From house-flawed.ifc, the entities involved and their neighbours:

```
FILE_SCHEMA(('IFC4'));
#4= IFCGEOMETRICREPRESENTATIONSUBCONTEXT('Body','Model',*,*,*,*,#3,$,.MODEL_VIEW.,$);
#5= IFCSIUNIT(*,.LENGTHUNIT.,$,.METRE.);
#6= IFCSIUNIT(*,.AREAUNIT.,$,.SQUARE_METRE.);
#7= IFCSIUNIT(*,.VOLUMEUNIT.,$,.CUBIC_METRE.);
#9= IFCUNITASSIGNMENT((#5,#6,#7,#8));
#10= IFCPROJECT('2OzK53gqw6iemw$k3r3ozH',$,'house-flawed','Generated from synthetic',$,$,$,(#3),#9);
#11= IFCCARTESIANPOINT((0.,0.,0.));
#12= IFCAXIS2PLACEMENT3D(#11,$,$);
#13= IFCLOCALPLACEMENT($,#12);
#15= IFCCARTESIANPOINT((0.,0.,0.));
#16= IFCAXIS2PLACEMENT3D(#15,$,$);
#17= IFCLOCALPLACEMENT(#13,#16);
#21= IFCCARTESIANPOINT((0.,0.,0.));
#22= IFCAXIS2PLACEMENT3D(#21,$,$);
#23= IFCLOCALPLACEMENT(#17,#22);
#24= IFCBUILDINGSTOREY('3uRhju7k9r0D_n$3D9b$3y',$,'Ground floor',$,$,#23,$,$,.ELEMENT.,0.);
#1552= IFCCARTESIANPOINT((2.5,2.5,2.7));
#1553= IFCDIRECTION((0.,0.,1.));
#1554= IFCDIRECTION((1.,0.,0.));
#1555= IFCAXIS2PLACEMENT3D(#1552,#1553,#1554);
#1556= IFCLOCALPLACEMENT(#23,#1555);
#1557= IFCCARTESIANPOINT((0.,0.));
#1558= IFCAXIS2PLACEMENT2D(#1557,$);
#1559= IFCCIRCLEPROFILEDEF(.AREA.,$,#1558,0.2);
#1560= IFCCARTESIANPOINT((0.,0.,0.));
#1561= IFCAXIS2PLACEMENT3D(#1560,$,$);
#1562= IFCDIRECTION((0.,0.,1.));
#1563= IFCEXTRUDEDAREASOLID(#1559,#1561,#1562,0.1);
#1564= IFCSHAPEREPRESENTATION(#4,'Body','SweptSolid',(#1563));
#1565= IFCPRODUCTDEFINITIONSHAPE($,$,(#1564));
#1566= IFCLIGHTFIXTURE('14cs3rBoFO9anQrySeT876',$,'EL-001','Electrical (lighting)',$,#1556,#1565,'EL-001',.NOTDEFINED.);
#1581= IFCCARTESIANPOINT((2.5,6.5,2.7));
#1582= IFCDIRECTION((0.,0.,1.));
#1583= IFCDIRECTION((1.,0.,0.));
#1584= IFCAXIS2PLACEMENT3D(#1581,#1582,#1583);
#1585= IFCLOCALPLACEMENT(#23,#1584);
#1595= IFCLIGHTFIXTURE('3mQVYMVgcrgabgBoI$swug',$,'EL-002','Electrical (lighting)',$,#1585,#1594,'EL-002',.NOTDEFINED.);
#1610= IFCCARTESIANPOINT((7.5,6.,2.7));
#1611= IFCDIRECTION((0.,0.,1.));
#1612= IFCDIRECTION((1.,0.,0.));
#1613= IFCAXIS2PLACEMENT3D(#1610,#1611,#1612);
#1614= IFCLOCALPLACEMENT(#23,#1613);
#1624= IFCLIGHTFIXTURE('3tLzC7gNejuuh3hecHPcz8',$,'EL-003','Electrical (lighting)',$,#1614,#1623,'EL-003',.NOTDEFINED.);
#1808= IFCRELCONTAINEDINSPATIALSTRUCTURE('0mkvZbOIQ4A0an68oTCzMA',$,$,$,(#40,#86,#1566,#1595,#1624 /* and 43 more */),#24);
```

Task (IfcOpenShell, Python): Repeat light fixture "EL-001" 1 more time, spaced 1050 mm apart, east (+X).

```python
import numpy as np
import ifcopenshell
import ifcopenshell.api.geometry
import ifcopenshell.api.root
import ifcopenshell.util.element
import ifcopenshell.util.placement

model = ifcopenshell.open("house-flawed.ifc")

source = model.by_guid("14cs3rBoFO9anQrySeT876")
base = ifcopenshell.util.placement.get_local_placement(source.ObjectPlacement)
step = np.array([1.0, 0.0, 0.0]) * 1.05

for i in range(1, 2):
    copy = ifcopenshell.api.root.copy_class(model, product=source)
    copy.Representation = ifcopenshell.util.element.copy_deep(
        model, source.Representation, exclude=["IfcGeometricRepresentationContext", "IfcRepresentationMap"]
    )
    copy.Tag = None
    matrix = base.copy()
    matrix[:3, 3] += i * step
    print("added at", matrix[:3, 3].round(3) + 0.0)
    ifcopenshell.api.geometry.edit_object_placement(model, product=copy, matrix=matrix, is_si=False)

model.write("house-flawed_updated.ifc")
```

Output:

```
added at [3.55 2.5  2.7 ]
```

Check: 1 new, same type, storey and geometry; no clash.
